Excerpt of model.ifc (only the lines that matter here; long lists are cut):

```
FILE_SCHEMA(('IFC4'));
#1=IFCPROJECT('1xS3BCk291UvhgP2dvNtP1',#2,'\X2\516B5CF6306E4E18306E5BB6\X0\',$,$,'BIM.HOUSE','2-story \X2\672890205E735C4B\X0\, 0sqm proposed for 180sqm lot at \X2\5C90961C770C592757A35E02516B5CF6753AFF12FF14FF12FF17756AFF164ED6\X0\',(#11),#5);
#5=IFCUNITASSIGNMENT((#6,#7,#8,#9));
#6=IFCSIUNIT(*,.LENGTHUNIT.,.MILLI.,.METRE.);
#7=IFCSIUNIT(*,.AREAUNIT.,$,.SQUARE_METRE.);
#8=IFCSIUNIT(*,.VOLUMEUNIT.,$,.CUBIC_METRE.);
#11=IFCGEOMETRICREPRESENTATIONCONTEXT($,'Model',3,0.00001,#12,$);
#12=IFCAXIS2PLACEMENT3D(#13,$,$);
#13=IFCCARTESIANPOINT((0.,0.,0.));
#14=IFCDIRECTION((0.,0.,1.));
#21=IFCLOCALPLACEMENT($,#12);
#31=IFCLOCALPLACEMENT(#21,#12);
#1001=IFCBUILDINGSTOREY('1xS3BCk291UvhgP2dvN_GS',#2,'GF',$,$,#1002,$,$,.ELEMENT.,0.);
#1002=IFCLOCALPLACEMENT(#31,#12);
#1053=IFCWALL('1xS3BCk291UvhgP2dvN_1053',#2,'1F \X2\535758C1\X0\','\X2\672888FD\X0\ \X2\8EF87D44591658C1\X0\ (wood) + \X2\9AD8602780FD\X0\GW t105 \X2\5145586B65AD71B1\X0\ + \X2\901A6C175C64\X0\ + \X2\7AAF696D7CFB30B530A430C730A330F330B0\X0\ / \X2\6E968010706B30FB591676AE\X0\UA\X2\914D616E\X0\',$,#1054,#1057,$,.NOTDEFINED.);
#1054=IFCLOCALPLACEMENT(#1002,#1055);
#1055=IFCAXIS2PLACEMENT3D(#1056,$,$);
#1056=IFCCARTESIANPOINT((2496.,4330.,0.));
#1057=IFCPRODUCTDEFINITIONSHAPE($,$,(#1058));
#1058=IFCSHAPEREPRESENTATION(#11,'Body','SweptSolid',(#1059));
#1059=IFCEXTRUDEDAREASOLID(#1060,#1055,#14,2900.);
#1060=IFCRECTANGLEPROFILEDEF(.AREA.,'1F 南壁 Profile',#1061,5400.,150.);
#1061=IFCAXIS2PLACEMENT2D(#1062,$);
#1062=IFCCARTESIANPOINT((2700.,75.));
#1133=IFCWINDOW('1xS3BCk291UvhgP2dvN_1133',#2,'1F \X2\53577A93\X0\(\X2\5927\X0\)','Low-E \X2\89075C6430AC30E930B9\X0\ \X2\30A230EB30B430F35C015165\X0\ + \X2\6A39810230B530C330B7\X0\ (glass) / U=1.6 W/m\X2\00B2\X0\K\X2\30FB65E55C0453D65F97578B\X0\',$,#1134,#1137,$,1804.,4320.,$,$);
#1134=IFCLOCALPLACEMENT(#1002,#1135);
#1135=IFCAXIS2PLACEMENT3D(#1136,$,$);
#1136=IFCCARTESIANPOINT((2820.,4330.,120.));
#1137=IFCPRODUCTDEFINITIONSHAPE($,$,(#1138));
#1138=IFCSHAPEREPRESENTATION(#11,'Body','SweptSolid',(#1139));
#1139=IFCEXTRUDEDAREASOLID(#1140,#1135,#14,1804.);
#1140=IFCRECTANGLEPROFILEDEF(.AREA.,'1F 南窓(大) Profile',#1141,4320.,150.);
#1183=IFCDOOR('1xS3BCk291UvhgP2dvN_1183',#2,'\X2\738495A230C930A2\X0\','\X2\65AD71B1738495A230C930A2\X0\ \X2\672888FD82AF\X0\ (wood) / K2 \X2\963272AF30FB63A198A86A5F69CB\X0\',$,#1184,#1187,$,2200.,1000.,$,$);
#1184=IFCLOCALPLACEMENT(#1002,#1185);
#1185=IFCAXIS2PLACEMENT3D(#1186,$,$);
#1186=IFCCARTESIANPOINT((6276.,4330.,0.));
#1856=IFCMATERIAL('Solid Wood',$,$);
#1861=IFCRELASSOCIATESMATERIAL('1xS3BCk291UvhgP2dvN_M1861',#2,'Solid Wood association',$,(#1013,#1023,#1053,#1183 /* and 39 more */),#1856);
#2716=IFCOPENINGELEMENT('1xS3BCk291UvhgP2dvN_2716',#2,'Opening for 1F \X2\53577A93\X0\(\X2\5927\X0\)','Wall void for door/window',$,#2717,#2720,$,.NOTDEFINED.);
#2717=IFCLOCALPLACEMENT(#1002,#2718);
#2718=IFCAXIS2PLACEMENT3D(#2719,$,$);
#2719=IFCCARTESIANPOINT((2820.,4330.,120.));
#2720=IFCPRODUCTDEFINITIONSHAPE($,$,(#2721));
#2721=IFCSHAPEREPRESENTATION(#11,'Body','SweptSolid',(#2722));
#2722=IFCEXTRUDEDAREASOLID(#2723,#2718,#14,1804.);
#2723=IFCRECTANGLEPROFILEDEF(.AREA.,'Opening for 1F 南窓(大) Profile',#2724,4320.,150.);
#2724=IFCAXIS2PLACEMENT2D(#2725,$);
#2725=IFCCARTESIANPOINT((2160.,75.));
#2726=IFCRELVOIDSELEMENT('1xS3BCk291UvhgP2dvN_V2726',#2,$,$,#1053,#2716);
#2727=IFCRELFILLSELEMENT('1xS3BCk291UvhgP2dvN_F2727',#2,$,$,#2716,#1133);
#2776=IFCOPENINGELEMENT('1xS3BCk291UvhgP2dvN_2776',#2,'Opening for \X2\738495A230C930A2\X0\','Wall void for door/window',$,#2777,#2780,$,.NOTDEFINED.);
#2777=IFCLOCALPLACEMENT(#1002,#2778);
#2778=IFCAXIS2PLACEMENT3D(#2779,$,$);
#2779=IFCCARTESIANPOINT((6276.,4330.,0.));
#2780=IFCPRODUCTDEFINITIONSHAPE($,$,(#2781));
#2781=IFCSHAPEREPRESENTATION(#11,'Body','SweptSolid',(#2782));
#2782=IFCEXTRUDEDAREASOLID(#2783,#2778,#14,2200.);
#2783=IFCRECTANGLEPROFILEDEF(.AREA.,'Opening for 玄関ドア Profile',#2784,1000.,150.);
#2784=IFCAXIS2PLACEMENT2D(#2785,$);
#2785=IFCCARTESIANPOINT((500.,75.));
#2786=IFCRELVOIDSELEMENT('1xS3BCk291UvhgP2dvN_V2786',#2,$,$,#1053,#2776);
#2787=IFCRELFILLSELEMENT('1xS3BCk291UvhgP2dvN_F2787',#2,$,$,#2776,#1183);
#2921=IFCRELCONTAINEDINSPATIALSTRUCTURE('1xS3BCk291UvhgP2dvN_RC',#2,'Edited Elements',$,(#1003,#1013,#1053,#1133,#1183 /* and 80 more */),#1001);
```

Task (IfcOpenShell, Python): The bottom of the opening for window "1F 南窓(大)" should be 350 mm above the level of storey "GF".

```python
import numpy as np
import ifcopenshell
import ifcopenshell.api.geometry
import ifcopenshell.geom
import ifcopenshell.util.element
import ifcopenshell.util.placement
import ifcopenshell.util.shape
import ifcopenshell.util.unit

model = ifcopenshell.open("model.ifc")
unit_scale = ifcopenshell.util.unit.calculate_unit_scale(model)

window = model.by_guid("1xS3BCk291UvhgP2dvN_1133")
opening = window.FillsVoids[0].RelatingOpeningElement
storey = ifcopenshell.util.element.get_container(window, ifc_class="IfcBuildingStorey")
level = ifcopenshell.util.placement.get_local_placement(storey.ObjectPlacement)[2, 3]

# The opening's origin need not be at the sill, so measure its lowest point.
shape = ifcopenshell.geom.create_shape(ifcopenshell.geom.settings(), opening)
bottom = ifcopenshell.util.shape.get_shape_bottom_elevation(shape, shape.geometry) / unit_scale
dz = level + 350.0 - bottom

shift = np.array([0.0, 0.0, dz])
# The window is not placed relative to its opening, so move both.
for product in (opening, window):
    matrix = ifcopenshell.util.placement.get_local_placement(product.ObjectPlacement)
    matrix[:3, 3] += shift
    ifcopenshell.api.geometry.edit_object_placement(model, product=product, matrix=matrix, is_si=False)

print(f"moved by {dz * unit_scale:+.3f} m")

model.write("model_v2.ifc")
```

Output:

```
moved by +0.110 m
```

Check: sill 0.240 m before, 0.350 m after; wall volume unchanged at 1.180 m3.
